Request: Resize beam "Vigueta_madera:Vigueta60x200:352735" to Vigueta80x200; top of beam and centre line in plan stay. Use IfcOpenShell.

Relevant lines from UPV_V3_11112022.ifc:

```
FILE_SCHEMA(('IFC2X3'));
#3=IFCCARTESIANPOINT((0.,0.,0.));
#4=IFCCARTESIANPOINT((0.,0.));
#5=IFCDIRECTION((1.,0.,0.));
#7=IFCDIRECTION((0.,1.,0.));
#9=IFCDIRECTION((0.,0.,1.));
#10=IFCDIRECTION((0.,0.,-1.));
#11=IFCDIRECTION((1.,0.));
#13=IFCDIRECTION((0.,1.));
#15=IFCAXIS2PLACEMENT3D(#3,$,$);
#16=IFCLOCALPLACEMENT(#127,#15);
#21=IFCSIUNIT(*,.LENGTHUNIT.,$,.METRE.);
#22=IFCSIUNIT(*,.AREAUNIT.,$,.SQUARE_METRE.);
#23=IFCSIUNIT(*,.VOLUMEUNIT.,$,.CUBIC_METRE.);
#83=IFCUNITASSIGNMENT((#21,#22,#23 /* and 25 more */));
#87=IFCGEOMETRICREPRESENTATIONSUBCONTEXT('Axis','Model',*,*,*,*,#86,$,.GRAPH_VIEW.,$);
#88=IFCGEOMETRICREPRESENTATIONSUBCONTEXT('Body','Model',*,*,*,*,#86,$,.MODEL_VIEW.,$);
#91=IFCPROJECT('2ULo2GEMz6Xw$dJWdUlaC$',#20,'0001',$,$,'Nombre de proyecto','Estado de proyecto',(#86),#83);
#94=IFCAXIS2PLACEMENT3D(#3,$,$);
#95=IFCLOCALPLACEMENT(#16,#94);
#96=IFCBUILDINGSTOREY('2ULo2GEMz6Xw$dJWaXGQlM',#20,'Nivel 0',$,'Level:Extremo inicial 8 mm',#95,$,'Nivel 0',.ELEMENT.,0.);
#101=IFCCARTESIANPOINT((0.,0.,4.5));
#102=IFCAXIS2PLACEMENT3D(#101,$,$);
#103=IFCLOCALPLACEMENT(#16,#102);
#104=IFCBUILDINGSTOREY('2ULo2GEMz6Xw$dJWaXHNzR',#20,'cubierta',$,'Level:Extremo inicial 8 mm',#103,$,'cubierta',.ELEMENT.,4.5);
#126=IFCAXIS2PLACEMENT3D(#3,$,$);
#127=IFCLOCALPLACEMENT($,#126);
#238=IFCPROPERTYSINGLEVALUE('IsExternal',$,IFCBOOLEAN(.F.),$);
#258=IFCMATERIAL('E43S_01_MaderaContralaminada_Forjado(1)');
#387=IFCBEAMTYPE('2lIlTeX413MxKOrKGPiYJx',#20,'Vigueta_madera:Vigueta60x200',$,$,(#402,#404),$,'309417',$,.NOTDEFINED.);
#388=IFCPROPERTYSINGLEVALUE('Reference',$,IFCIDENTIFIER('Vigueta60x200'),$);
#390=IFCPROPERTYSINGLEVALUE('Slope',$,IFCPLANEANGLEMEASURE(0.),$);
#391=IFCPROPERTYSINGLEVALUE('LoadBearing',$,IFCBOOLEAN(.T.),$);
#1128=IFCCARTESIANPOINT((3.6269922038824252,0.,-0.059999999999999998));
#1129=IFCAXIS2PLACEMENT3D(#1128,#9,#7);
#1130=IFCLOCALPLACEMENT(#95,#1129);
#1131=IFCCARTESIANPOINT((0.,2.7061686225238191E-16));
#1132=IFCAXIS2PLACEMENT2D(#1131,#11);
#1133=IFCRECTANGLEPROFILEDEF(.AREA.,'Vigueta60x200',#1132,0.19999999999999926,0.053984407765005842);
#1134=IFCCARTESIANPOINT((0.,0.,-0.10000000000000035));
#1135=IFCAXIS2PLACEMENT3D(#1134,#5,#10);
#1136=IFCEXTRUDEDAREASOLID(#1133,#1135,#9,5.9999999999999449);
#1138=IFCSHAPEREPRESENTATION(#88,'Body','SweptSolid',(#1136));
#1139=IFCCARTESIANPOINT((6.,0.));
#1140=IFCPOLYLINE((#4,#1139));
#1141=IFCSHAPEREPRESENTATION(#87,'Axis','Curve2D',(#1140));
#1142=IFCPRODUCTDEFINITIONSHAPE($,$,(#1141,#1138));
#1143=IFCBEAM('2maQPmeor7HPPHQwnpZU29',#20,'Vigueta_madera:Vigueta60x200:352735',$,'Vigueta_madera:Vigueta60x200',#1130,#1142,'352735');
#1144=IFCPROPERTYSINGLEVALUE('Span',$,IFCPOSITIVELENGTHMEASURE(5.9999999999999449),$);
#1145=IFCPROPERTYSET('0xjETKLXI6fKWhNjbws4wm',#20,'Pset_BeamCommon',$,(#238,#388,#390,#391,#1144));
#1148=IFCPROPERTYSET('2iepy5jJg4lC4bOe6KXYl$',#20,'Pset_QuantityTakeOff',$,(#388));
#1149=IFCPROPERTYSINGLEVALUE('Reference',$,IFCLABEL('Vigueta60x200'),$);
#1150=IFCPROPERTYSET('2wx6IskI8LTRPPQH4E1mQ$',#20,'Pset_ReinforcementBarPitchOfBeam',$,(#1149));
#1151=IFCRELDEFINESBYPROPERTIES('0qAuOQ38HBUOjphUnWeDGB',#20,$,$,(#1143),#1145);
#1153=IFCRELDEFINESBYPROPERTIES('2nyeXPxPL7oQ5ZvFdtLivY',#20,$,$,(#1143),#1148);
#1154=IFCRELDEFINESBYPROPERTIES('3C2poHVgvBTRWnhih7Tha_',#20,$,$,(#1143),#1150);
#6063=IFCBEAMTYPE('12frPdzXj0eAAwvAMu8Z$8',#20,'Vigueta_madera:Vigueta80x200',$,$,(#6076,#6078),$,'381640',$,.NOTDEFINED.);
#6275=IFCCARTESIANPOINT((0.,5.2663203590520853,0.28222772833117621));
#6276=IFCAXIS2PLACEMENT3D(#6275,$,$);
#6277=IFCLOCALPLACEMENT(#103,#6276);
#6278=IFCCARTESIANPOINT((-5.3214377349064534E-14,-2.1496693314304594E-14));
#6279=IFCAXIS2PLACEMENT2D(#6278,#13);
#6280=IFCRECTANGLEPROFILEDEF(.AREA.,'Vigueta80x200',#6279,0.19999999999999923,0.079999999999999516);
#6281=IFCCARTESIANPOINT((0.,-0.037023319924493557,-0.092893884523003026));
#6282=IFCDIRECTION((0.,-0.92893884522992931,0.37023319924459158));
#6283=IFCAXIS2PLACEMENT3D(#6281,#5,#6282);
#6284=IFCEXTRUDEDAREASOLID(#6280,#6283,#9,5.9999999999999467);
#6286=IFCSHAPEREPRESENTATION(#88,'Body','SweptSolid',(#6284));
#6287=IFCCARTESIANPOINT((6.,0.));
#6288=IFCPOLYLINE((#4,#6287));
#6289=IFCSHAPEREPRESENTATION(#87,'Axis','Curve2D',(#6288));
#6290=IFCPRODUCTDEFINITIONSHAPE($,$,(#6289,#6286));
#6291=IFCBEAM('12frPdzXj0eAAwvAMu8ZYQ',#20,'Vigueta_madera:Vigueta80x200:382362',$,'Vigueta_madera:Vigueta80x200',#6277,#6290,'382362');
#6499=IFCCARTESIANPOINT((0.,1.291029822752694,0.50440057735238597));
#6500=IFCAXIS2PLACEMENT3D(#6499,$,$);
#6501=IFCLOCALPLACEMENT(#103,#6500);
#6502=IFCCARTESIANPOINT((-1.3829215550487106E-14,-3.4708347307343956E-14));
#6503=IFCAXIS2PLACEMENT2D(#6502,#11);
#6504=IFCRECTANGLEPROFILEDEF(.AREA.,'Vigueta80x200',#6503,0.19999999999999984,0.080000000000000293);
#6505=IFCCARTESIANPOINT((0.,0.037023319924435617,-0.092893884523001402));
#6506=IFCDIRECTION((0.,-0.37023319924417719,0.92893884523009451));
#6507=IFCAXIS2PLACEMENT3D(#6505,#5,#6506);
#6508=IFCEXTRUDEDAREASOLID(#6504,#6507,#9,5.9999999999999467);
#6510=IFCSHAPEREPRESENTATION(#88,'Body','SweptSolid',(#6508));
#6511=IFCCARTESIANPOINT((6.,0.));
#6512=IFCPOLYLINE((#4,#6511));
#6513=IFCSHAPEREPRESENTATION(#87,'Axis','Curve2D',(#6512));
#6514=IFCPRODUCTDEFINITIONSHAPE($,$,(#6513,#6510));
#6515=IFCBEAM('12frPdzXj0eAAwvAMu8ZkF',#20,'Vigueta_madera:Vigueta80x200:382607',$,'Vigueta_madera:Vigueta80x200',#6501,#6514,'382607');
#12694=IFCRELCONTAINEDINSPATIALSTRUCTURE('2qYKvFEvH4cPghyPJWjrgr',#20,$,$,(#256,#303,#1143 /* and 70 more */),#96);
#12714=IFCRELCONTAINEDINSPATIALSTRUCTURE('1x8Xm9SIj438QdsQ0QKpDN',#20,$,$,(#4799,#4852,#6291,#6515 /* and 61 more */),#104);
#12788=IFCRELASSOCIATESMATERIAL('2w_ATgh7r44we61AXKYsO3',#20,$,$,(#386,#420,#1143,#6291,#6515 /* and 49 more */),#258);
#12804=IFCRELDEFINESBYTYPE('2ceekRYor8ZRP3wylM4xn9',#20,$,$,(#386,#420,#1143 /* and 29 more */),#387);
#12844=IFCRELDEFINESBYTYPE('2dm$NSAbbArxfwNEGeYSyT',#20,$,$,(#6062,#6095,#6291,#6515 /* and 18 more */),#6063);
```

```python
import ifcopenshell
import ifcopenshell.api.pset
import ifcopenshell.api.type
import ifcopenshell.util.element
import ifcopenshell.util.representation

model = ifcopenshell.open("UPV_V3_11112022.ifc")

member = model.by_id(1143)
source = next(p for p in model.by_type("IfcRectangleProfileDef") if p.ProfileName == "Vigueta80x200")

body = ifcopenshell.util.representation.get_representation(member, "Model", "Body")
solid = body.Items[0]
old_profile = solid.SweptArea

# Copy the section's sizes but keep this member's own profile position.
profile = ifcopenshell.util.element.copy(model, source)
# Profiles are centred, so shift by half the change in depth to hold the top.
shift = (old_profile.XDim - profile.XDim) / 2
x, y = old_profile.Position.Location.Coordinates
up = (-1.0, 0.0)  # upwards, in the solid's own plane
location = model.createIfcCartesianPoint((x + up[0] * shift, y + up[1] * shift))
profile.Position = model.createIfcAxis2Placement2D(location, old_profile.Position.RefDirection)
solid.SweptArea = profile
if not model.get_total_inverses(old_profile):
    ifcopenshell.util.element.remove_deep2(model, old_profile)

new_type = model.by_guid("12frPdzXj0eAAwvAMu8Z$8")
ifcopenshell.api.type.assign_type(
    model, related_objects=[member], relating_type=new_type, should_map_representations=False
)
member.Name = member.Name.replace("Vigueta60x200", "Vigueta80x200")
member.ObjectType = "Vigueta_madera:Vigueta80x200"
pset = model.by_id(ifcopenshell.util.element.get_pset(member, "Pset_BeamCommon", should_inherit=False)["id"])
ifcopenshell.api.pset.edit_pset(model, pset=pset, properties={"Reference": "Vigueta80x200"})
pset = model.by_id(ifcopenshell.util.element.get_pset(member, "Pset_QuantityTakeOff", should_inherit=False)["id"])
ifcopenshell.api.pset.edit_pset(model, pset=pset, properties={"Reference": "Vigueta80x200"})
pset = model.by_id(ifcopenshell.util.element.get_pset(member, "Pset_ReinforcementBarPitchOfBeam", should_inherit=False)["id"])
ifcopenshell.api.pset.edit_pset(model, pset=pset, properties={"Reference": "Vigueta80x200"})

print(solid.SweptArea)

model.write("UPV_V3_11112022_edited.ifc")
```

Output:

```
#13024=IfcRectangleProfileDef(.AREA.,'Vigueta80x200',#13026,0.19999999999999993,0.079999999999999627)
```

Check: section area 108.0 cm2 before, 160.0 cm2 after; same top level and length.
